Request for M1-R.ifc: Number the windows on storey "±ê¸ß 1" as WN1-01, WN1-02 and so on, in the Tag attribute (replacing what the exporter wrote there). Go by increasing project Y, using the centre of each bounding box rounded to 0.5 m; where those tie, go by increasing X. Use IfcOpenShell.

First a look at what the model holds.

```python
import ifcopenshell
import ifcopenshell.util.element
import ifcopenshell.util.placement

model = ifcopenshell.open("M1-R.ifc")
print(model.schema)
storey = next(s for s in model.by_type("IfcBuildingStorey") if s.Name == "±ê¸ß 1")
windows = [e for e in ifcopenshell.util.element.get_decomposition(storey) if e.is_a("IfcWindow")]
for e in sorted(windows, key=lambda e: e.id()):
    origin = ifcopenshell.util.placement.get_local_placement(e.ObjectPlacement)[:3, 3]
    print(e.id(), e.Tag, e.Name, origin.round(2) + 0.0, sep=" | ")
```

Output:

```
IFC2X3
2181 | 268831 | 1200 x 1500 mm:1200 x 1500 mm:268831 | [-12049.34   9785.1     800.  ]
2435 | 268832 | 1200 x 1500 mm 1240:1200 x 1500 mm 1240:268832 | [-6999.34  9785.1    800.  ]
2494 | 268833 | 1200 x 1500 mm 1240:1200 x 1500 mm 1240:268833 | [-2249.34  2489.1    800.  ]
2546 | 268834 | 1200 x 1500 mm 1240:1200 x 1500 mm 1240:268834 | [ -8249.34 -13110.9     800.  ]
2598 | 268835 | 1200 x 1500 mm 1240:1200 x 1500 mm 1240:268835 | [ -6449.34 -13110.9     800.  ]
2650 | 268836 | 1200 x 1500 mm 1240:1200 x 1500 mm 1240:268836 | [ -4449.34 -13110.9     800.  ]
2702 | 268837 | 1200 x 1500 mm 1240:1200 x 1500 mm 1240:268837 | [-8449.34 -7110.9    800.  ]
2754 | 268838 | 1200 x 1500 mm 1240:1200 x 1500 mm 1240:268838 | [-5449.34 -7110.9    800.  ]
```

```python
import ifcopenshell
import ifcopenshell.geom
import ifcopenshell.util.element
import ifcopenshell.util.shape

model = ifcopenshell.open("M1-R.ifc")
settings = ifcopenshell.geom.settings()
settings.set("use-world-coords", True)


def centre(element):
    shape = ifcopenshell.geom.create_shape(settings, element)
    return ifcopenshell.util.shape.get_bbox_centroid(shape.geometry)


storey = next(s for s in model.by_type("IfcBuildingStorey") if s.Name == "±ê¸ß 1")
windows = [e for e in ifcopenshell.util.element.get_decomposition(storey) if e.is_a("IfcWindow")]

# Insertion points can sit at a corner or the storey origin, so sort by the geometry (in metres).
centres = {e: centre(e) for e in windows}
windows.sort(key=lambda e: (round(centres[e][1] / 0.5), centres[e][0]))

for i, e in enumerate(windows, start=1):
    number = f"WN1-{i:02d}"
    e.Tag = number
    print(e.id(), number)

model.write("M1-R_rev.ifc")
```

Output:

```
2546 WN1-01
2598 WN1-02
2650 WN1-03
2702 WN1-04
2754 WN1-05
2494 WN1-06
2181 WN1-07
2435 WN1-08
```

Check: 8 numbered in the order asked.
